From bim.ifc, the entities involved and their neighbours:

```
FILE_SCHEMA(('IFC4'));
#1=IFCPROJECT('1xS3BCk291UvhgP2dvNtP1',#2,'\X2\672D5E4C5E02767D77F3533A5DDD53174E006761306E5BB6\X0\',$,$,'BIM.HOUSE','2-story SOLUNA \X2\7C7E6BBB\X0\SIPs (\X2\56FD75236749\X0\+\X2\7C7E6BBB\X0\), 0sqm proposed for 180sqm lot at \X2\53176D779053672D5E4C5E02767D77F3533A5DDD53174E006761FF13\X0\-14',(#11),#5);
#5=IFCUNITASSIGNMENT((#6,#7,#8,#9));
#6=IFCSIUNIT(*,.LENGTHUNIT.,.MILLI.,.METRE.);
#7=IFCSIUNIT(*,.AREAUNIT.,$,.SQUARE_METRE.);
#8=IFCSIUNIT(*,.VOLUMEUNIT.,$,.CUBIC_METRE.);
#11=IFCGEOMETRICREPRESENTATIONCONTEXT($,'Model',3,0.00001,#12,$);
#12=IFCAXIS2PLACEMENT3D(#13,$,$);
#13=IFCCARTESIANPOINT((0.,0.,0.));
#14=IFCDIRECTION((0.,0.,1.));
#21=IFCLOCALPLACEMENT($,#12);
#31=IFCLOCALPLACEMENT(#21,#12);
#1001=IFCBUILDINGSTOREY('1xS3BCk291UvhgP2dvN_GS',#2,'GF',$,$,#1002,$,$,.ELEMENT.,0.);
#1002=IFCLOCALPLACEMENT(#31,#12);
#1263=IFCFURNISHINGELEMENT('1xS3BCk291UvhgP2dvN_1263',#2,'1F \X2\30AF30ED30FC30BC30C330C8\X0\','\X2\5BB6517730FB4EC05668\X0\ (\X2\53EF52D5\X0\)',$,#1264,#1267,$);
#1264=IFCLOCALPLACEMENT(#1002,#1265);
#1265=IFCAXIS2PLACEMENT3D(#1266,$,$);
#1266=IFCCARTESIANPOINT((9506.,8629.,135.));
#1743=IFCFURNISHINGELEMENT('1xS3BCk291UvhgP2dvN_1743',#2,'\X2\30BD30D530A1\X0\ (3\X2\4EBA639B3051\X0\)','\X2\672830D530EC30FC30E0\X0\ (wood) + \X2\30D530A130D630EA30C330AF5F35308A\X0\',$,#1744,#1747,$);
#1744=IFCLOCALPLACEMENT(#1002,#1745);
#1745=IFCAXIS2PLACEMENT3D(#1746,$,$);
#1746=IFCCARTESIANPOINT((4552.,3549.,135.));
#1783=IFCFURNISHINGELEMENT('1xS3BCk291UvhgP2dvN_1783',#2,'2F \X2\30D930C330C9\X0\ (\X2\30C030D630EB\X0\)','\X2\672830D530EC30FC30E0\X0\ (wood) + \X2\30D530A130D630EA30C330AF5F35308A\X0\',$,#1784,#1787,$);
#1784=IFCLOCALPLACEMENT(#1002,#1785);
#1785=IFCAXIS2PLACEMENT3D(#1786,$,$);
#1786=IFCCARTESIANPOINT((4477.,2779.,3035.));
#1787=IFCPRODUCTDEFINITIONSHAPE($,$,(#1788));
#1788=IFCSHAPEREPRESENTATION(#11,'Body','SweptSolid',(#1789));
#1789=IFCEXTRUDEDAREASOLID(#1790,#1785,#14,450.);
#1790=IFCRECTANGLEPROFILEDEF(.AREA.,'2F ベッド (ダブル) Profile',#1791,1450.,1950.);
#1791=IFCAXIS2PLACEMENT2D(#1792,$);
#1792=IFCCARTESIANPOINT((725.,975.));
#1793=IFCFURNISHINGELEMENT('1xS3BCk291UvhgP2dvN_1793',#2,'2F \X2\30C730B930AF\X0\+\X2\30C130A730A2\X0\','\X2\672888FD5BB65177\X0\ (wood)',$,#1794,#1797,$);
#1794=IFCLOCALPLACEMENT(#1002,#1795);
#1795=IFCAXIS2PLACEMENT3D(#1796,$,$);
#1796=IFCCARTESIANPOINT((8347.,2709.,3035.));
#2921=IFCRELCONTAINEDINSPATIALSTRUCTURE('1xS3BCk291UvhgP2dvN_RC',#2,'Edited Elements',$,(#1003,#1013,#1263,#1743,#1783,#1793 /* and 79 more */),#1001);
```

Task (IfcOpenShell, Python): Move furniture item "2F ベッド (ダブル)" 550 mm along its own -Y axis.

```python
import ifcopenshell
import ifcopenshell.api.geometry
import ifcopenshell.util.placement

model = ifcopenshell.open("bim.ifc")

item = model.by_guid("1xS3BCk291UvhgP2dvN_1783")
matrix = ifcopenshell.util.placement.get_local_placement(item.ObjectPlacement)
matrix[:3, 3] -= matrix[:3, 1] * 550.0
ifcopenshell.api.geometry.edit_object_placement(model, product=item, matrix=matrix, is_si=False)

print(ifcopenshell.util.placement.get_local_placement(item.ObjectPlacement).round(3) + 0.0)

model.write("bim_edited.ifc")
```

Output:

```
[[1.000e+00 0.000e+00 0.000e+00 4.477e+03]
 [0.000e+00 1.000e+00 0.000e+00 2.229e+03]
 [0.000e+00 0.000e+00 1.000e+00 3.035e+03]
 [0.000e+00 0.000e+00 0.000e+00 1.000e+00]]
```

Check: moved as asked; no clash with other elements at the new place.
